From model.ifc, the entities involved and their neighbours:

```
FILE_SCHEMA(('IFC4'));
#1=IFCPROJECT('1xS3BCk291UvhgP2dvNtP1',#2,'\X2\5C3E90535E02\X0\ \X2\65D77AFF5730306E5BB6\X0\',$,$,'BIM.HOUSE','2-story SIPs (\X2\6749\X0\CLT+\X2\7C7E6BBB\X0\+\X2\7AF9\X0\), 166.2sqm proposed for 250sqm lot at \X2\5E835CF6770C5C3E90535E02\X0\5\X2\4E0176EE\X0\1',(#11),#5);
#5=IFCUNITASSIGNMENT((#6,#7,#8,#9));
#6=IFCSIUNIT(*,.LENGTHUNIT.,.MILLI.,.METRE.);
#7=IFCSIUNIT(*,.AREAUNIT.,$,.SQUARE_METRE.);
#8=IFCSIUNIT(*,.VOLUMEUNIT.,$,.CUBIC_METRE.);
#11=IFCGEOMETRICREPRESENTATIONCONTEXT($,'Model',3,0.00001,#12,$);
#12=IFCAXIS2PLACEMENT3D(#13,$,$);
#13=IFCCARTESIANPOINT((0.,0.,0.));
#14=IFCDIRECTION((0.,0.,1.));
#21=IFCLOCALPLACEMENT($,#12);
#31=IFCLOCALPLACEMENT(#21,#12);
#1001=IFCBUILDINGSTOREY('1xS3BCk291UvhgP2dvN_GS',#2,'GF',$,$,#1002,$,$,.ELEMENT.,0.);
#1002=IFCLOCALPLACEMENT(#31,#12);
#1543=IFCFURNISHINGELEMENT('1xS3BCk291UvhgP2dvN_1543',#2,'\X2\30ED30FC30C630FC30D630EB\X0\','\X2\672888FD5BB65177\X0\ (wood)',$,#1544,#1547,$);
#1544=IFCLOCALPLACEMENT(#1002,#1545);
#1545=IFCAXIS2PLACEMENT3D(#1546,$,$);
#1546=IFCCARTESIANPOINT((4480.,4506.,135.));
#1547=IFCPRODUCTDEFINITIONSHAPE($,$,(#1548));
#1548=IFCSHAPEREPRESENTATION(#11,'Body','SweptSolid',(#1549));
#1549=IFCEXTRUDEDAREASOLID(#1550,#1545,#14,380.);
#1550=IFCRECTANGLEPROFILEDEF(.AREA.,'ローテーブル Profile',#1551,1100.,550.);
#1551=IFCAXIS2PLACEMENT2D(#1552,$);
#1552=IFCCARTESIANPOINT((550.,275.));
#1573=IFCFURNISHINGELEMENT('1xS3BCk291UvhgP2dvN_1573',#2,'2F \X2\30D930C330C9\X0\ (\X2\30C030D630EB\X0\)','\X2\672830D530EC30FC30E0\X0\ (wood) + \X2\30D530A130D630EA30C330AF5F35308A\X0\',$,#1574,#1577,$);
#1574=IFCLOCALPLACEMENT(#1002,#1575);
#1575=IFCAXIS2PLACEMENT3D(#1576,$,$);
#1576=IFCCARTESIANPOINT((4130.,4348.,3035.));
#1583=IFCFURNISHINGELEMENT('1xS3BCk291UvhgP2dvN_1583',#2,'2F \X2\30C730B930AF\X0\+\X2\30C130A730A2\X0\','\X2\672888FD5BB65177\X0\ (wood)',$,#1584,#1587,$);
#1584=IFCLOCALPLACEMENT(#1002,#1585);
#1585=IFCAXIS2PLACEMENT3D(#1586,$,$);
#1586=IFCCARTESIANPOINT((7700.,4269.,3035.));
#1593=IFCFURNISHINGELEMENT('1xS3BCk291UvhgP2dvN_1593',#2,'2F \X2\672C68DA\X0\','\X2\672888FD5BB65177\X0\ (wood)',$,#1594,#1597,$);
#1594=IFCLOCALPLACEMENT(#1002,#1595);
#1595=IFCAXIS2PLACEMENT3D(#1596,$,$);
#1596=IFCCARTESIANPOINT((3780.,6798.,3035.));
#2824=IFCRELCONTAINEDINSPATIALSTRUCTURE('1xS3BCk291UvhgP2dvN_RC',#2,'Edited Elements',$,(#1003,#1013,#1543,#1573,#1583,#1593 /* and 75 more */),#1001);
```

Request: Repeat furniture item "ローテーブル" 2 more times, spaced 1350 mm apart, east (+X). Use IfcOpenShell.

```python
import numpy as np
import ifcopenshell
import ifcopenshell.api.geometry
import ifcopenshell.api.root
import ifcopenshell.util.element
import ifcopenshell.util.placement

model = ifcopenshell.open("model.ifc")


def reuse_history(source, copy):
    """copy_class also copies each property set's owner history, people and application; keep the originals."""
    for rel in copy.IsDefinedBy:
        if rel.is_a("IfcRelDefinesByProperties") and (history := rel.RelatingPropertyDefinition.OwnerHistory):
            rel.RelatingPropertyDefinition.OwnerHistory = source.OwnerHistory
            ifcopenshell.util.element.remove_deep2(model, history)


source = model.by_guid("1xS3BCk291UvhgP2dvN_1543")
base = ifcopenshell.util.placement.get_local_placement(source.ObjectPlacement)
step = np.array([1.0, 0.0, 0.0]) * 1350.0

for i in range(1, 3):
    copy = ifcopenshell.api.root.copy_class(model, product=source)
    copy.Representation = ifcopenshell.util.element.copy_deep(
        model, source.Representation, exclude=["IfcGeometricRepresentationContext", "IfcRepresentationMap"]
    )
    reuse_history(source, copy)
    matrix = base.copy()
    matrix[:3, 3] += i * step
    print("added at", matrix[:3, 3].round(3) + 0.0)
    ifcopenshell.api.geometry.edit_object_placement(model, product=copy, matrix=matrix, is_si=False)

model.write("model-out.ifc")
```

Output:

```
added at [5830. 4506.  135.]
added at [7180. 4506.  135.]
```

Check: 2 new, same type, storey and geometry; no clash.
